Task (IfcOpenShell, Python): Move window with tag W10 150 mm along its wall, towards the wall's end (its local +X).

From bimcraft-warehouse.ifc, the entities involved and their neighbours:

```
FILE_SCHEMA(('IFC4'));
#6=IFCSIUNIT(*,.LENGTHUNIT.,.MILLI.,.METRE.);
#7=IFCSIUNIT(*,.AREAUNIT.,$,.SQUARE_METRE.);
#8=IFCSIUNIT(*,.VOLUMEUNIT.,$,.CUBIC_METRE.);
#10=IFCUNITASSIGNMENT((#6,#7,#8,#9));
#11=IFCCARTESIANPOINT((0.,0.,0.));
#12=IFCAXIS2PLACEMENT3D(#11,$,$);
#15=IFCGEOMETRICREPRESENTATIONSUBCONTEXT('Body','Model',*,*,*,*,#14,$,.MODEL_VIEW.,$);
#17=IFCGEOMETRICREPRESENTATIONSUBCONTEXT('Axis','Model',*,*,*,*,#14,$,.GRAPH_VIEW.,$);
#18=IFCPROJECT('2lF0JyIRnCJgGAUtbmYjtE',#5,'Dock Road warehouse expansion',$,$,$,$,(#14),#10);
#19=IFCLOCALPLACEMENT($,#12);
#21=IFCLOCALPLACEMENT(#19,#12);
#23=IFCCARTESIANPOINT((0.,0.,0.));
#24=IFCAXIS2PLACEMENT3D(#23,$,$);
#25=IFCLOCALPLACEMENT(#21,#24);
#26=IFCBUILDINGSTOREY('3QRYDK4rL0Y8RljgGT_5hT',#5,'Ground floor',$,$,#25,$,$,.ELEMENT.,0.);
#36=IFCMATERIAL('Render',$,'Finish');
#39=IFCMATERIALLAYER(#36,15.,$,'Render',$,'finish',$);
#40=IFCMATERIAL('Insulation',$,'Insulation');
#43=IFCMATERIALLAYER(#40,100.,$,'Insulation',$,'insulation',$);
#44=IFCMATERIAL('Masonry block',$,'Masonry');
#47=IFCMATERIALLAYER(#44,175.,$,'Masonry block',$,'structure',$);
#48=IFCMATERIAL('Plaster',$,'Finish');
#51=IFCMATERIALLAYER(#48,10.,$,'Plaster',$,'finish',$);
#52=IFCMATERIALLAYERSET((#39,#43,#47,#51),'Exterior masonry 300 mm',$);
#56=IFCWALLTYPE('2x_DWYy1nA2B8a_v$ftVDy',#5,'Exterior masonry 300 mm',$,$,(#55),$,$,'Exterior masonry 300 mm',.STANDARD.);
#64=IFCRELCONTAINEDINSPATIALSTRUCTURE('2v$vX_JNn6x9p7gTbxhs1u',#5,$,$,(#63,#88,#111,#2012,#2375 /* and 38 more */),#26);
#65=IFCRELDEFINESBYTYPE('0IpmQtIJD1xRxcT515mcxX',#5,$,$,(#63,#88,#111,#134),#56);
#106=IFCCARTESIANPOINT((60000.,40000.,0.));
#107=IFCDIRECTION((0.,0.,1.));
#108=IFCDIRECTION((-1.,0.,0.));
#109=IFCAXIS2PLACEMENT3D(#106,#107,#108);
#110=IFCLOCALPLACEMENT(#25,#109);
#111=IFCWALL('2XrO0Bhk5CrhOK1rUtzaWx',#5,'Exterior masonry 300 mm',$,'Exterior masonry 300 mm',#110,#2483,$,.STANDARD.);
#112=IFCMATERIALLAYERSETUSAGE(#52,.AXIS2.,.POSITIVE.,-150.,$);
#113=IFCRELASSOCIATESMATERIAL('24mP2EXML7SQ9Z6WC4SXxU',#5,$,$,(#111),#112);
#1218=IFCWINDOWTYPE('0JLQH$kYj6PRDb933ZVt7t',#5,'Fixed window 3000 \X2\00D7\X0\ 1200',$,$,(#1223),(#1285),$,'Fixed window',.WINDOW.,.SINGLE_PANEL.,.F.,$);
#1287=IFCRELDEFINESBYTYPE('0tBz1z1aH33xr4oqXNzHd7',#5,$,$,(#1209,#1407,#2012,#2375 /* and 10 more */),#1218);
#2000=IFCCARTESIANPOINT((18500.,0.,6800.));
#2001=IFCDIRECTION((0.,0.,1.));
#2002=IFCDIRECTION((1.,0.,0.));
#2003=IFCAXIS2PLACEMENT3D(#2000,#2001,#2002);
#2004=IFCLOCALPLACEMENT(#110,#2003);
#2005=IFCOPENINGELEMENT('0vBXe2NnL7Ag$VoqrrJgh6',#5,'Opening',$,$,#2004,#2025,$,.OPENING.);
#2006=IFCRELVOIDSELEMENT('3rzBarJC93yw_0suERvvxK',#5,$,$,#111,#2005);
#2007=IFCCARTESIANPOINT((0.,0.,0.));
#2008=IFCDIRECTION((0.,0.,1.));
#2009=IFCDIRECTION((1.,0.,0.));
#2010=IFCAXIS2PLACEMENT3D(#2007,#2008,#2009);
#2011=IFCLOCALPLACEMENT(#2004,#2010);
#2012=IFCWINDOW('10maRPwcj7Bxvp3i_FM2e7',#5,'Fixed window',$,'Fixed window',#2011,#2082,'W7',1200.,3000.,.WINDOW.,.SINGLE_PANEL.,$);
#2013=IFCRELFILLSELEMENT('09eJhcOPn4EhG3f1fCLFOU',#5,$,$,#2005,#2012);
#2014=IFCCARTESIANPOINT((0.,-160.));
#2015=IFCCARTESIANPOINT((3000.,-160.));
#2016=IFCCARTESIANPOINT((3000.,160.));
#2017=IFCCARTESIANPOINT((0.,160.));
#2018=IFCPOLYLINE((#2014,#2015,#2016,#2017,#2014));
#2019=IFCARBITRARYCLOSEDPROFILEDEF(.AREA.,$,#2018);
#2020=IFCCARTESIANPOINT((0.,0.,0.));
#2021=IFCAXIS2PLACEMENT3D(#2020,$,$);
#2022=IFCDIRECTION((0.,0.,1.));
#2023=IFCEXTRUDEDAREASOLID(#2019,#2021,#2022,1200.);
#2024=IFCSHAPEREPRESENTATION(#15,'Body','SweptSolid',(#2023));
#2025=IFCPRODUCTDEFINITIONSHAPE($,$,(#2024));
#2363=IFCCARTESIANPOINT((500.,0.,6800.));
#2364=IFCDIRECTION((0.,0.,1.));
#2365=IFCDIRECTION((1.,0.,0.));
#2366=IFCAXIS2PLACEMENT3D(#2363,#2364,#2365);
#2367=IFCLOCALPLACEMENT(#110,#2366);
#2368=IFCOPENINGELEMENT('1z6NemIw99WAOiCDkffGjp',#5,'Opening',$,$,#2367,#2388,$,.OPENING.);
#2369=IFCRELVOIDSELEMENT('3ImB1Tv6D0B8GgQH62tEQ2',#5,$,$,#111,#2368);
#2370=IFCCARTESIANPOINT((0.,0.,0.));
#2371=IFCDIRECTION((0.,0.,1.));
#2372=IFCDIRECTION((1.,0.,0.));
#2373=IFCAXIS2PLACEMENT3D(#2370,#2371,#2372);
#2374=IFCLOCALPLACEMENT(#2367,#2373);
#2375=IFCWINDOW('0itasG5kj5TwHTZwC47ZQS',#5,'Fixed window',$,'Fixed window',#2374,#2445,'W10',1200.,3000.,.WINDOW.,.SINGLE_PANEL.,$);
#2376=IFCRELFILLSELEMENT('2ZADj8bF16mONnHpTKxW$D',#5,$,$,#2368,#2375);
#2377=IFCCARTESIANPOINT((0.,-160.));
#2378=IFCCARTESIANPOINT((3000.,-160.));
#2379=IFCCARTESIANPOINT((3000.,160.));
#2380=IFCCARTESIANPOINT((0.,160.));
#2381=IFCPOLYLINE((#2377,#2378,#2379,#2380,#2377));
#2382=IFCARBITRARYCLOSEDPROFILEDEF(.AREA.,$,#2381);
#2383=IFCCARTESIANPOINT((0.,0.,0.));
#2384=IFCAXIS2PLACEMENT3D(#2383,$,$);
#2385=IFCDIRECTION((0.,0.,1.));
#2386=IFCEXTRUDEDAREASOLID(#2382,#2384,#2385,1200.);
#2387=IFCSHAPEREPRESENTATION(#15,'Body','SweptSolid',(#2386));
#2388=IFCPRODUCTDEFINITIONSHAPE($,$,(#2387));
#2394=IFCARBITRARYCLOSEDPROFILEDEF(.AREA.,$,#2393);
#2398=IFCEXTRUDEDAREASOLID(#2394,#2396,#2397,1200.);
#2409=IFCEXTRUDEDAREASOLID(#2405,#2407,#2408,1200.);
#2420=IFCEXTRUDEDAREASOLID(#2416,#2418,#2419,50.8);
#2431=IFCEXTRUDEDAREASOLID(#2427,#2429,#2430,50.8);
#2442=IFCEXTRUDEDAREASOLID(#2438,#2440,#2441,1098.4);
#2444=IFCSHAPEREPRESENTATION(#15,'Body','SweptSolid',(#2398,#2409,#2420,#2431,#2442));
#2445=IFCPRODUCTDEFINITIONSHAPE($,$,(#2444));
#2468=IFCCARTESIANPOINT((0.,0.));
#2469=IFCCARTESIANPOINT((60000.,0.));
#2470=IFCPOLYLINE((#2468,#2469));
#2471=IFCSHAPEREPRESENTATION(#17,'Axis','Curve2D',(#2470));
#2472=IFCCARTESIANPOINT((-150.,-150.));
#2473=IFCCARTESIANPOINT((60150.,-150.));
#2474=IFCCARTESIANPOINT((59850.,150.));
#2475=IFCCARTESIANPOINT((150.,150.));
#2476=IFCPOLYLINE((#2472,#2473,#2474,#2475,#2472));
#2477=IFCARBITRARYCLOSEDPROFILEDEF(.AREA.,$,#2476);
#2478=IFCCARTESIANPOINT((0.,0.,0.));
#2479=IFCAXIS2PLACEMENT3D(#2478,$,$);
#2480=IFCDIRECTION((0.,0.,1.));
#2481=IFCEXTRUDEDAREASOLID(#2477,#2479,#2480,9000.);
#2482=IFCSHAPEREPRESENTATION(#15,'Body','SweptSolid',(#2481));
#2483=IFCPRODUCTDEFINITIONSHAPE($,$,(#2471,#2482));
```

```python
import ifcopenshell
import ifcopenshell.api.geometry
import ifcopenshell.util.placement
import ifcopenshell.util.unit

model = ifcopenshell.open("bimcraft-warehouse.ifc")
unit_scale = ifcopenshell.util.unit.calculate_unit_scale(model)

window = model.by_guid("0itasG5kj5TwHTZwC47ZQS")
opening = window.FillsVoids[0].RelatingOpeningElement
wall = opening.VoidsElements[0].RelatingBuildingElement

wall_matrix = ifcopenshell.util.placement.get_local_placement(wall.ObjectPlacement)
shift = wall_matrix[:3, 0] * 0.15 / unit_scale
before = ifcopenshell.util.placement.get_local_placement(window.ObjectPlacement)[:3, 3].copy()

# The window is placed relative to its opening, so it follows when the opening moves.
matrix = ifcopenshell.util.placement.get_local_placement(opening.ObjectPlacement)
matrix[:3, 3] += shift
ifcopenshell.api.geometry.edit_object_placement(
    model, product=opening, matrix=matrix, is_si=False, should_transform_children=True
)

after = ifcopenshell.util.placement.get_local_placement(window.ObjectPlacement)[:3, 3]
print("window moved by", (after - before).round(3) + 0.0)

model.write("bimcraft-warehouse-out.ifc")
```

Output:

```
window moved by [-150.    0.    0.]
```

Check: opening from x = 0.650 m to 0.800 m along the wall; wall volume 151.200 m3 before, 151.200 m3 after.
